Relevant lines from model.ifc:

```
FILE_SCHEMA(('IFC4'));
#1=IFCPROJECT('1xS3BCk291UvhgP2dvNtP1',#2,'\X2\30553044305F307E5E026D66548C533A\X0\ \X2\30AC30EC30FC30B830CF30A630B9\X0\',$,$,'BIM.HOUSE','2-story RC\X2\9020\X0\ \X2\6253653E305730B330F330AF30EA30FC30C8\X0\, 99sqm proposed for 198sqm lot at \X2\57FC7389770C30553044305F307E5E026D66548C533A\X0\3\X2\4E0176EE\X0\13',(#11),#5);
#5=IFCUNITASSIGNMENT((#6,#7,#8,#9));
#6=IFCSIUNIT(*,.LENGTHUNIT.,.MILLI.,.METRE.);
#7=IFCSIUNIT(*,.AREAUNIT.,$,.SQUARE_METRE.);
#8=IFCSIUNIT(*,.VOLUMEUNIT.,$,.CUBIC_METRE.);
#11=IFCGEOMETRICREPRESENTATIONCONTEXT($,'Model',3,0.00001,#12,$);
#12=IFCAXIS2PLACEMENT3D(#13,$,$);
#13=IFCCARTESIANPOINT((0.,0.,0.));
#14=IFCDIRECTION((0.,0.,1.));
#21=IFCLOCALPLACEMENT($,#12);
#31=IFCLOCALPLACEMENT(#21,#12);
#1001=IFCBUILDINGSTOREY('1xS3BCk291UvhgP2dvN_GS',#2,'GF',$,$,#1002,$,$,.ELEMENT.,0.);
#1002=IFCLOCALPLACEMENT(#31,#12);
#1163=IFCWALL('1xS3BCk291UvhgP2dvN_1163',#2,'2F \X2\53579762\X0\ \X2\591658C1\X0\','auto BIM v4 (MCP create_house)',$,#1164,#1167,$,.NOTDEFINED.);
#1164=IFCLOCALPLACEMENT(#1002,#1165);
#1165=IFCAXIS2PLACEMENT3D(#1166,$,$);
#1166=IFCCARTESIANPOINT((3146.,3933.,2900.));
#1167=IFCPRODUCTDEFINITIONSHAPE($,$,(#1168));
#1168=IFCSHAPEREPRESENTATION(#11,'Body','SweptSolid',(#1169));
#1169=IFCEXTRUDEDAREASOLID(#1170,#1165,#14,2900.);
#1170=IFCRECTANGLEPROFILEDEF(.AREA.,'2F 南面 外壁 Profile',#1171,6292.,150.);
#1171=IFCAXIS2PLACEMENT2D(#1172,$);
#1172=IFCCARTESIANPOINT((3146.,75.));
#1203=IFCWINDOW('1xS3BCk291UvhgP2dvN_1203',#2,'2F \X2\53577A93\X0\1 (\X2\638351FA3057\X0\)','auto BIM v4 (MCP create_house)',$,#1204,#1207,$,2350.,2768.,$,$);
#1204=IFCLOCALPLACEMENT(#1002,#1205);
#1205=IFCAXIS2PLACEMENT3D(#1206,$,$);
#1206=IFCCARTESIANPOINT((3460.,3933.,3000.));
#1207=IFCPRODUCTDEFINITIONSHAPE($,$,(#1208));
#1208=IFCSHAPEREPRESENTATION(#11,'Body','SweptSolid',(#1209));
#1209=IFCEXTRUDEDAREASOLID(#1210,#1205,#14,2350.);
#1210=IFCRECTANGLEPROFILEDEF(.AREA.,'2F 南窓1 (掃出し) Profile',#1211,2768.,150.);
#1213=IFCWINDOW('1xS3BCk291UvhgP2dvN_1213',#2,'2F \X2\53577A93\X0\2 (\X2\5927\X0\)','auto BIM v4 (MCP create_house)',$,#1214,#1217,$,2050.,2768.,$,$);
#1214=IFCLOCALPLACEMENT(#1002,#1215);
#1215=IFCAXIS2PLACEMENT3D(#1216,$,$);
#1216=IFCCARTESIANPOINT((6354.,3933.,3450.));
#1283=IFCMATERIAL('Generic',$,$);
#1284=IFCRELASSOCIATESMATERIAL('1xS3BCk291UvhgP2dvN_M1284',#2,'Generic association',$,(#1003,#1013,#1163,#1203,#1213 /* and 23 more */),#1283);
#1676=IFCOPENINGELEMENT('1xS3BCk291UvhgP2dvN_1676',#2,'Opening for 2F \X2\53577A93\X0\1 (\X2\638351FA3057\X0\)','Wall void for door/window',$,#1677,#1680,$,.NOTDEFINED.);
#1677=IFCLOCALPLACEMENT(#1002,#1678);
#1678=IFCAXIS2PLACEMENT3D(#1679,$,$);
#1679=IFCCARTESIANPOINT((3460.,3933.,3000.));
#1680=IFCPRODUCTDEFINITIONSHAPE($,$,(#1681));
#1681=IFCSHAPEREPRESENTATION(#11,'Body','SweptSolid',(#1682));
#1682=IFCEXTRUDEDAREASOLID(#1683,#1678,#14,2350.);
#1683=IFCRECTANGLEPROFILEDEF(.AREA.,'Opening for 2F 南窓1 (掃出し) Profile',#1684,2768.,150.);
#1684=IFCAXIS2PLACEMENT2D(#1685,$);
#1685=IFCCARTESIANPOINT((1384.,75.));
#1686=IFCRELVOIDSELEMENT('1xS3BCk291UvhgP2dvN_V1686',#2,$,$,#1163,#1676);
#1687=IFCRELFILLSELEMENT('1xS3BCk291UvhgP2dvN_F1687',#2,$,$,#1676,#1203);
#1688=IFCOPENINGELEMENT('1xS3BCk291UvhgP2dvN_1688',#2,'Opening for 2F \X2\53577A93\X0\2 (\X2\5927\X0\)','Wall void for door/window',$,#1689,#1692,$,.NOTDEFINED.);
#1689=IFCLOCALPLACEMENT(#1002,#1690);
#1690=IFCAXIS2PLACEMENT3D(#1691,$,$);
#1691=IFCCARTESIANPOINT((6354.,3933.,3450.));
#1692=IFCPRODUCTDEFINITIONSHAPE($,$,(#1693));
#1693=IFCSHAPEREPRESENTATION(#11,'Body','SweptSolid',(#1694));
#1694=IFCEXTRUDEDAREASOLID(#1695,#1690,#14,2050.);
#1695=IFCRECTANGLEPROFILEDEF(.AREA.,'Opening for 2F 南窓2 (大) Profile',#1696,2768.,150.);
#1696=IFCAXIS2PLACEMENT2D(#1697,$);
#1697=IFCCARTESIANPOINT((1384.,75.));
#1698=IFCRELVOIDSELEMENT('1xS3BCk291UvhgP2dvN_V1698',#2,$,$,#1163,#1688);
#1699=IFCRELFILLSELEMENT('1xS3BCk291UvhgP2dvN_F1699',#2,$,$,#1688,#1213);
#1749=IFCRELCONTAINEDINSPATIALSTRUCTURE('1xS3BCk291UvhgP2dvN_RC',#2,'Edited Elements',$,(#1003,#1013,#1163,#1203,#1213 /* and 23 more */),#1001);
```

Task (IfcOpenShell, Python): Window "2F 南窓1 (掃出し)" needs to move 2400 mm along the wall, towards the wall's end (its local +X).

```python
import ifcopenshell
import ifcopenshell.api.geometry
import ifcopenshell.util.placement

model = ifcopenshell.open("model.ifc")

window = model.by_id(1203)
opening = window.FillsVoids[0].RelatingOpeningElement
wall = opening.VoidsElements[0].RelatingBuildingElement

wall_matrix = ifcopenshell.util.placement.get_local_placement(wall.ObjectPlacement)
shift = wall_matrix[:3, 0] * 2400.0
before = ifcopenshell.util.placement.get_local_placement(window.ObjectPlacement)[:3, 3].copy()

# The window is not placed relative to its opening, so move both.
for product in (opening, window):
    matrix = ifcopenshell.util.placement.get_local_placement(product.ObjectPlacement)
    matrix[:3, 3] += shift
    ifcopenshell.api.geometry.edit_object_placement(model, product=product, matrix=matrix, is_si=False)

after = ifcopenshell.util.placement.get_local_placement(window.ObjectPlacement)[:3, 3]
print("window moved by", (after - before).round(3) + 0.0)

model.write("model_updated.ifc")
```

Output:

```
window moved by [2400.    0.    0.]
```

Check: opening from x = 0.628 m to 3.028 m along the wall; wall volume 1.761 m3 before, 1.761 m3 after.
